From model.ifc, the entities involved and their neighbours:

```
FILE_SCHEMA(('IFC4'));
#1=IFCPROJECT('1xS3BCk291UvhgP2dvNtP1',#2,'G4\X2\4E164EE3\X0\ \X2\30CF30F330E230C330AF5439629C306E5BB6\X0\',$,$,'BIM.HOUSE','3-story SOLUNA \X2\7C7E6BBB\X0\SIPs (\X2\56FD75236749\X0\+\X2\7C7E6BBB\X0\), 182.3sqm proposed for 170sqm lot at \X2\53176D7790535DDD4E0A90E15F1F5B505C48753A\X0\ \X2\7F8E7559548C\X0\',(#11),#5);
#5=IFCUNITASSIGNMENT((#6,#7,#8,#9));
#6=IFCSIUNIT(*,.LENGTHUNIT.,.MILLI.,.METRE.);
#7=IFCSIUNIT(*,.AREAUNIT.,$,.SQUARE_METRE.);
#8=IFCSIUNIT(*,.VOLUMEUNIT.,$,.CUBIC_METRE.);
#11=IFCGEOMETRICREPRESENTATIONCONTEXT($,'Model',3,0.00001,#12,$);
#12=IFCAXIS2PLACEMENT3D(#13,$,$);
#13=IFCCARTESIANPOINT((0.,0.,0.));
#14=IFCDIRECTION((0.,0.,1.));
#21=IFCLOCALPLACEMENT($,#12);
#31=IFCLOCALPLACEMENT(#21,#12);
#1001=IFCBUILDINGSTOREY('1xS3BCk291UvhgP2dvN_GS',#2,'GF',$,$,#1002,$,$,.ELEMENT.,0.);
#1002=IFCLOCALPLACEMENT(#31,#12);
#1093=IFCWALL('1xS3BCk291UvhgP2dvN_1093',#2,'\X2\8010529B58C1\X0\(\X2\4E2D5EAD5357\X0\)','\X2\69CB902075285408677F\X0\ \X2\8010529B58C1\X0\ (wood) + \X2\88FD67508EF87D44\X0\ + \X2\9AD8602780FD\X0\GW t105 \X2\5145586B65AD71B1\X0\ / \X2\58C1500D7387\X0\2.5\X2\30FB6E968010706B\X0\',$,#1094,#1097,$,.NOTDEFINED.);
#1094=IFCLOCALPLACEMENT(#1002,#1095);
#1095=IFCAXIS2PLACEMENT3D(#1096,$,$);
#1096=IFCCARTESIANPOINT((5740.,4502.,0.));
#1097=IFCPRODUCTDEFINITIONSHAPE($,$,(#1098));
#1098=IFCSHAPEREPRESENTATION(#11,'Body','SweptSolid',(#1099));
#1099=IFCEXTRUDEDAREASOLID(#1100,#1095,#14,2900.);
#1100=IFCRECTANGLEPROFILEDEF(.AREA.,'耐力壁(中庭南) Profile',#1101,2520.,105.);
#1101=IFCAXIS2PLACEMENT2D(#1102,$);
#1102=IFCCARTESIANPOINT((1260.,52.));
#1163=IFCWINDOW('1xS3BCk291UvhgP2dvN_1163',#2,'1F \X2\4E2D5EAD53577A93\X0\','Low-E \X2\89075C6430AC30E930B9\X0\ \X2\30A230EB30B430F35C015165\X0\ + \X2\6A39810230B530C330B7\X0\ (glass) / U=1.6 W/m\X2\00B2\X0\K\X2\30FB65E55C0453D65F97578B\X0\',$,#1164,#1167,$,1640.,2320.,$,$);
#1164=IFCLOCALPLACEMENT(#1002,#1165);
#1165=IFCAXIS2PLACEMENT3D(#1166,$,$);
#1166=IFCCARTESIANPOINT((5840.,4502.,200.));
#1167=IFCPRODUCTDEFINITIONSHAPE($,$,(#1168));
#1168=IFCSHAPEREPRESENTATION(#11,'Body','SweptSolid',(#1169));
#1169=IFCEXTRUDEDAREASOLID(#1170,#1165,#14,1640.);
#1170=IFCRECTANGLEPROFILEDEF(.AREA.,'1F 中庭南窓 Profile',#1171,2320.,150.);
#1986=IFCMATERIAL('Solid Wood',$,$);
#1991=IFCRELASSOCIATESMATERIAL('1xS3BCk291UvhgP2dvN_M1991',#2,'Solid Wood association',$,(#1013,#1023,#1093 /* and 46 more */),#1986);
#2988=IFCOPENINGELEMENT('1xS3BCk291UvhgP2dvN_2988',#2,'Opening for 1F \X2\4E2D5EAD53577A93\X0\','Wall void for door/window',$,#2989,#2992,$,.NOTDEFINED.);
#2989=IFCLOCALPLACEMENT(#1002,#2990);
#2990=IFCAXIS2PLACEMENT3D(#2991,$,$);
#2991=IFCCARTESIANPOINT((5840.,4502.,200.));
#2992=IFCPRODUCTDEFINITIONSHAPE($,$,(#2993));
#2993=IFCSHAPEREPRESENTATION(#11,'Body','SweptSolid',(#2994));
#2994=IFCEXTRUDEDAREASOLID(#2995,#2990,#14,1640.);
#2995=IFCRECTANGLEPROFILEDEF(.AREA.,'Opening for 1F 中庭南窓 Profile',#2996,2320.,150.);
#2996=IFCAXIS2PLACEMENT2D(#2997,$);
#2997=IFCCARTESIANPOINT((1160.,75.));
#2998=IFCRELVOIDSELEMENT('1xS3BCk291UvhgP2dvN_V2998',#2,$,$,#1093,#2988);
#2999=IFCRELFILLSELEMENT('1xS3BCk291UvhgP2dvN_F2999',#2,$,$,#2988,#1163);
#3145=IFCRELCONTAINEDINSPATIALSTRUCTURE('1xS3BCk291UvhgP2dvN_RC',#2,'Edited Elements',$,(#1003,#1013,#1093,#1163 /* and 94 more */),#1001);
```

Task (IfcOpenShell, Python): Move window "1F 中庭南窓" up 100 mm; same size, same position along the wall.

```python
import numpy as np
import ifcopenshell
import ifcopenshell.api.geometry
import ifcopenshell.util.placement
import ifcopenshell.util.unit

model = ifcopenshell.open("model.ifc")
unit_scale = ifcopenshell.util.unit.calculate_unit_scale(model)

window = model.by_guid("1xS3BCk291UvhgP2dvN_1163")
opening = window.FillsVoids[0].RelatingOpeningElement
dz = 0.1 / unit_scale

shift = np.array([0.0, 0.0, dz])
# The window is not placed relative to its opening, so move both.
for product in (opening, window):
    matrix = ifcopenshell.util.placement.get_local_placement(product.ObjectPlacement)
    matrix[:3, 3] += shift
    ifcopenshell.api.geometry.edit_object_placement(model, product=product, matrix=matrix, is_si=False)

print(f"moved by {dz * unit_scale:+.3f} m")

model.write("model_edited.ifc")
```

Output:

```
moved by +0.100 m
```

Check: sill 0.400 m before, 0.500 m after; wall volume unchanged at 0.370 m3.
